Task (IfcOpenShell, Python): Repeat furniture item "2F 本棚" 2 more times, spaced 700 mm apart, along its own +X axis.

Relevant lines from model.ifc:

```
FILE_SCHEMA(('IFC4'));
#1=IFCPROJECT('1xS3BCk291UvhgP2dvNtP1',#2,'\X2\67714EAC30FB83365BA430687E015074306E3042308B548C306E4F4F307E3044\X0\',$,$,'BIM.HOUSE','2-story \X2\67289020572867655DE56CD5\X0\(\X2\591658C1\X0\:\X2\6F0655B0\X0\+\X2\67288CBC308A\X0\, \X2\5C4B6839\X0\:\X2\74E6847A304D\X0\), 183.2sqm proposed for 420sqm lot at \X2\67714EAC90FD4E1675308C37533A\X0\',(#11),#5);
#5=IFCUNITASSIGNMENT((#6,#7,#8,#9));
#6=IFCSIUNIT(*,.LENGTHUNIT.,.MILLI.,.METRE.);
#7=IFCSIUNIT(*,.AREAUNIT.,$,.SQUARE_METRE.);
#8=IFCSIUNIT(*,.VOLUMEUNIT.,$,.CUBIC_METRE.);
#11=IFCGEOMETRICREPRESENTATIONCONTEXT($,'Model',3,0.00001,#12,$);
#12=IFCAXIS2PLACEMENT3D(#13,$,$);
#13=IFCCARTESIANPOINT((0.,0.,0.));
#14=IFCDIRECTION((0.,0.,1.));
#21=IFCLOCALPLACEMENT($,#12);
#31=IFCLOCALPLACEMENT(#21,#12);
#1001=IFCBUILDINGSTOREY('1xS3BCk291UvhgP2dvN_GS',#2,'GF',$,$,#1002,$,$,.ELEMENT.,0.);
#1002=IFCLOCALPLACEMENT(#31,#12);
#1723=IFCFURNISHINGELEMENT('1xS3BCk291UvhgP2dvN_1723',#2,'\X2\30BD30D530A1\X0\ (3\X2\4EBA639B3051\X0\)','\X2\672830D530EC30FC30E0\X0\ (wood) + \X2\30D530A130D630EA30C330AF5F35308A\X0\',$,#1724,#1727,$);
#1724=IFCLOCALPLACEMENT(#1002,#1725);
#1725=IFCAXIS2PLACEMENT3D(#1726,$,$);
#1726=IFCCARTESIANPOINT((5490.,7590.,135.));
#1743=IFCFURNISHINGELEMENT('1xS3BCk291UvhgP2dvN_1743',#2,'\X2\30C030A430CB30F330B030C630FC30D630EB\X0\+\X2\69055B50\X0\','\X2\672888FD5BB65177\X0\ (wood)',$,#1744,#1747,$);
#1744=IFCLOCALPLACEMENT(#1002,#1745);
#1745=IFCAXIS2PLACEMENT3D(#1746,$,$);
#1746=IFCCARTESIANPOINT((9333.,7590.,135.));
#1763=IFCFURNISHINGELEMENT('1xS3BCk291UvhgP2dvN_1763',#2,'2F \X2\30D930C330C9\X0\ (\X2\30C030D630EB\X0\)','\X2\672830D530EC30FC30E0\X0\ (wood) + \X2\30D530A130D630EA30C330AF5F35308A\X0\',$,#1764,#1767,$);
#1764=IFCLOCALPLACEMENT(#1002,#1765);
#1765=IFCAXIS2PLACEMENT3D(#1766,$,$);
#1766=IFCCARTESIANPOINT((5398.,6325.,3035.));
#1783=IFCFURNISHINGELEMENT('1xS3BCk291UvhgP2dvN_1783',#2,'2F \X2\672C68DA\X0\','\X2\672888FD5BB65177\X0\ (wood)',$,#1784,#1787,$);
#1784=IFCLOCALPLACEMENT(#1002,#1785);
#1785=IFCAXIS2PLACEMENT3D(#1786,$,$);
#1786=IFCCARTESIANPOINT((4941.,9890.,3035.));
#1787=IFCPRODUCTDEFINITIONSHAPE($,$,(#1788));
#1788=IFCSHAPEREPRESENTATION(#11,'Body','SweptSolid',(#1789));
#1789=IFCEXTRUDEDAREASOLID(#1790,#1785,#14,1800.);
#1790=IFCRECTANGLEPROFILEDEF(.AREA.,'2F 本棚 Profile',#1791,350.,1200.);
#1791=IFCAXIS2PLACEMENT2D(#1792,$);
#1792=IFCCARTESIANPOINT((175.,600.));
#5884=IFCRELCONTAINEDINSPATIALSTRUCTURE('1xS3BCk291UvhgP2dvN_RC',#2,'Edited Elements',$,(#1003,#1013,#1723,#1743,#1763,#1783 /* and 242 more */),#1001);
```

```python
import ifcopenshell
import ifcopenshell.api.geometry
import ifcopenshell.api.root
import ifcopenshell.util.element
import ifcopenshell.util.placement
import ifcopenshell.util.unit

model = ifcopenshell.open("model.ifc")
unit_scale = ifcopenshell.util.unit.calculate_unit_scale(model)


def reuse_history(source, copy):
    """copy_class also copies each property set's owner history, people and application; keep the originals."""
    for rel in copy.IsDefinedBy:
        if rel.is_a("IfcRelDefinesByProperties") and (history := rel.RelatingPropertyDefinition.OwnerHistory):
            rel.RelatingPropertyDefinition.OwnerHistory = source.OwnerHistory
            ifcopenshell.util.element.remove_deep2(model, history)


source = model.by_id(1783)
base = ifcopenshell.util.placement.get_local_placement(source.ObjectPlacement)
step = base[:3, 0] * 0.7 / unit_scale

for i in range(1, 3):
    copy = ifcopenshell.api.root.copy_class(model, product=source)
    copy.Representation = ifcopenshell.util.element.copy_deep(
        model, source.Representation, exclude=["IfcGeometricRepresentationContext", "IfcRepresentationMap"]
    )
    reuse_history(source, copy)
    matrix = base.copy()
    matrix[:3, 3] += i * step
    print("added at", matrix[:3, 3].round(3) + 0.0)
    ifcopenshell.api.geometry.edit_object_placement(model, product=copy, matrix=matrix, is_si=False)

model.write("model_edited.ifc")
```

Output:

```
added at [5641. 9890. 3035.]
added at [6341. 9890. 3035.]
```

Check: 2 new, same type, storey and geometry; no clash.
